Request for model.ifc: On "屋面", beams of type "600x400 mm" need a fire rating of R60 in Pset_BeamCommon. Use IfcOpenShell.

First a look at what the model holds.

```python
import ifcopenshell
import ifcopenshell.util.element

model = ifcopenshell.open("model.ifc")
print(model.schema)
storey = next(s for s in model.by_type("IfcBuildingStorey") if s.Name == "屋面")
beams = [e for e in ifcopenshell.util.element.get_decomposition(storey) if e.is_a("IfcBeam")]
seen = {}
for e in beams:
    element_type = ifcopenshell.util.element.get_type(e)
    key = (element_type.Name if element_type != e and element_type else None, ifcopenshell.util.element.get_pset(e, "Pset_BeamCommon", "FireRating"))
    seen[key] = seen.get(key, 0) + 1
for (name, value), count in sorted(seen.items(), key=str):
    print(count, "x", name, "|", value)
```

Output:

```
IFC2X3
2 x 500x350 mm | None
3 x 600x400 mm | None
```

```python
import ifcopenshell
import ifcopenshell.api.pset
import ifcopenshell.util.element

model = ifcopenshell.open("model.ifc")

storey = next(s for s in model.by_type("IfcBuildingStorey") if s.Name == "屋面")
beams = [e for e in ifcopenshell.util.element.get_decomposition(storey) if e.is_a("IfcBeam")]

count = 0
for e in beams:
    element_type = ifcopenshell.util.element.get_type(e)
    if element_type in (None, e) or element_type.Name != "600x400 mm":
        continue
    # add_pset returns the element's existing set when there is one.
    pset = ifcopenshell.api.pset.add_pset(model, product=e, name="Pset_BeamCommon")
    ifcopenshell.api.pset.edit_pset(model, pset=pset, properties={"FireRating": "R60"})
    count += 1

print(count, "beams updated")

model.write("model_edited.ifc")
```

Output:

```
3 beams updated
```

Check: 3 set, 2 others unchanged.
